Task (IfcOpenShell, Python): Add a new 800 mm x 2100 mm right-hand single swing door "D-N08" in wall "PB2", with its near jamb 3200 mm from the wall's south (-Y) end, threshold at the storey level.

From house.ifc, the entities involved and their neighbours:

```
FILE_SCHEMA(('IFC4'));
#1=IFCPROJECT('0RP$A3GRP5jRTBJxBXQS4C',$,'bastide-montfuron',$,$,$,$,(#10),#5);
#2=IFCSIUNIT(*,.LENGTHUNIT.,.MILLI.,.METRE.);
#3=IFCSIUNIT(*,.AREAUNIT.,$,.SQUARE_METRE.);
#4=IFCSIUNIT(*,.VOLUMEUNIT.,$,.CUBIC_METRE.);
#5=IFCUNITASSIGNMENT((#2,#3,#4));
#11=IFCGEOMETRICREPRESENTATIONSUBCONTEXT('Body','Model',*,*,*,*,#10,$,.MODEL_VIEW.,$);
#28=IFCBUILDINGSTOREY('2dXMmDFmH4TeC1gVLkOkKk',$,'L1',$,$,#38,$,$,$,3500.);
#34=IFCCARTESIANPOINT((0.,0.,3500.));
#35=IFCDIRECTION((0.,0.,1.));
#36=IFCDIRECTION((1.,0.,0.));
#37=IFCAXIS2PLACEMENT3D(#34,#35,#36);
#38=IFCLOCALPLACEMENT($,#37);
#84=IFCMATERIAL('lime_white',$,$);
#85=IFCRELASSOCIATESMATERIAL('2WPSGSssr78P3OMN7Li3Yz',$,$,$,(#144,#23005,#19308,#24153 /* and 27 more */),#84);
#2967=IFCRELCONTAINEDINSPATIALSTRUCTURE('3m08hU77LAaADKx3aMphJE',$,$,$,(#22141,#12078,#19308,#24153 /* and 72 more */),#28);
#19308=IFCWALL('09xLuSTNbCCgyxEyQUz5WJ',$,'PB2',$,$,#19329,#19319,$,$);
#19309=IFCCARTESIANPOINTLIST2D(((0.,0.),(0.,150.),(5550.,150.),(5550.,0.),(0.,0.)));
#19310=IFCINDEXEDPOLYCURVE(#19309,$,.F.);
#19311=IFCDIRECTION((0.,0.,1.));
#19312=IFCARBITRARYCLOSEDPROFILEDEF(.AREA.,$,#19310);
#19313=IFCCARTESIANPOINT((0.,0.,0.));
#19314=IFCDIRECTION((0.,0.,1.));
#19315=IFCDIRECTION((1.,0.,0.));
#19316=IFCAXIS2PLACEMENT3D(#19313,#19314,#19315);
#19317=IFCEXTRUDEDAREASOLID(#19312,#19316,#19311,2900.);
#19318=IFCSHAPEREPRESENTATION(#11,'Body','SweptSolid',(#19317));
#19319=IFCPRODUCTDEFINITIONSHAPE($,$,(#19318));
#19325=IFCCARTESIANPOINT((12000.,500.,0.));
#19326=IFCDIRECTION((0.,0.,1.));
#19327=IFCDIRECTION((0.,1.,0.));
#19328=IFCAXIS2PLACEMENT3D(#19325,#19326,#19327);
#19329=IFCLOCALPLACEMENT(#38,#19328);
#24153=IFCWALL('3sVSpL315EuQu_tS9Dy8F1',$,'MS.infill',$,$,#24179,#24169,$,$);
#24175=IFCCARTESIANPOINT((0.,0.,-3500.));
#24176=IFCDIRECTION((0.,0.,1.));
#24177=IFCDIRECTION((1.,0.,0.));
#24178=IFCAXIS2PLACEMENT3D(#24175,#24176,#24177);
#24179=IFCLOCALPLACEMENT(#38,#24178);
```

```python
import numpy as np
import ifcopenshell
import ifcopenshell.api.feature
import ifcopenshell.api.geometry
import ifcopenshell.api.root
import ifcopenshell.api.spatial
import ifcopenshell.geom
import ifcopenshell.util.element
import ifcopenshell.util.placement
import ifcopenshell.util.representation
import ifcopenshell.util.shape
import ifcopenshell.util.unit

model = ifcopenshell.open("house.ifc")
unit_scale = ifcopenshell.util.unit.calculate_unit_scale(model)
settings = ifcopenshell.geom.settings()


def volume(element):
    """Net volume in cubic metres, openings subtracted."""
    shape = ifcopenshell.geom.create_shape(settings, element)
    return ifcopenshell.util.shape.get_volume(shape.geometry)


wall = model.by_id(19308)
storey = ifcopenshell.util.element.get_container(wall, ifc_class="IfcBuildingStorey")
context = ifcopenshell.util.representation.get_context(model, "Model", "Body", "MODEL_VIEW")
before = volume(wall)

width, height, from_end, sill = 0.8, 2.1, 3.2, 0.0  # metres

# The wall runs along its own X axis, and the end named is its -X end.
wall_shape = ifcopenshell.geom.create_shape(settings, wall)
x, y, z = ifcopenshell.util.shape.get_vertices(wall_shape.geometry).T
start = x.min() + from_end
face, thickness = float(y.min()), float(y.max() - y.min())
wall_matrix = ifcopenshell.util.placement.get_local_placement(wall.ObjectPlacement)
level = ifcopenshell.util.placement.get_local_placement(storey.ObjectPlacement)[2, 3]


def in_wall(x, y):
    """Placement at x, y metres in the wall's axes, at sill height."""
    matrix = wall_matrix.copy()
    matrix[:, 3] = wall_matrix @ np.array([x / unit_scale, y / unit_scale, 0.0, 1.0])
    matrix[2, 3] = level + sill / unit_scale
    return matrix


# Opening: a box that overshoots both wall faces by 50 mm.
opening = ifcopenshell.api.root.create_entity(model, ifc_class="IfcOpeningElement", predefined_type="OPENING")
box = ifcopenshell.api.geometry.add_wall_representation(
    model, context=context, length=width, height=height, thickness=thickness + 0.1
)
ifcopenshell.api.geometry.assign_representation(model, product=opening, representation=box)
ifcopenshell.api.geometry.edit_object_placement(model, product=opening, matrix=in_wall(start, face - 0.05), is_si=False)
ifcopenshell.api.feature.add_feature(model, feature=opening, element=wall)

door = ifcopenshell.api.root.create_entity(model, ifc_class="IfcDoor", name="D-N08", predefined_type="DOOR")
door.OverallWidth, door.OverallHeight = width / unit_scale, height / unit_scale
door.OperationType = "SINGLE_SWING_RIGHT"
body = ifcopenshell.api.geometry.add_door_representation(
    model,
    context=context,
    overall_width=door.OverallWidth,
    overall_height=door.OverallHeight,
    operation_type="SINGLE_SWING_RIGHT",
    lining_properties={"LiningDepth": thickness / unit_scale, "ThresholdDepth": thickness / unit_scale},
)
ifcopenshell.api.geometry.assign_representation(model, product=door, representation=body)
ifcopenshell.api.spatial.assign_container(model, products=[door], relating_structure=storey)
ifcopenshell.api.feature.add_filling(model, opening=opening, element=door)

# The lining spans the wall, so the door starts at the wall face.
ifcopenshell.api.geometry.edit_object_placement(model, product=door, matrix=in_wall(start, face), is_si=False)

after = volume(wall)

print(f"wall volume {before:.3f} -> {after:.3f} m3")

model.write("house-out.ifc")
```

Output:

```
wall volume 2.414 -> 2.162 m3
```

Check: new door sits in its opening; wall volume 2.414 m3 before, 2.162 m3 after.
